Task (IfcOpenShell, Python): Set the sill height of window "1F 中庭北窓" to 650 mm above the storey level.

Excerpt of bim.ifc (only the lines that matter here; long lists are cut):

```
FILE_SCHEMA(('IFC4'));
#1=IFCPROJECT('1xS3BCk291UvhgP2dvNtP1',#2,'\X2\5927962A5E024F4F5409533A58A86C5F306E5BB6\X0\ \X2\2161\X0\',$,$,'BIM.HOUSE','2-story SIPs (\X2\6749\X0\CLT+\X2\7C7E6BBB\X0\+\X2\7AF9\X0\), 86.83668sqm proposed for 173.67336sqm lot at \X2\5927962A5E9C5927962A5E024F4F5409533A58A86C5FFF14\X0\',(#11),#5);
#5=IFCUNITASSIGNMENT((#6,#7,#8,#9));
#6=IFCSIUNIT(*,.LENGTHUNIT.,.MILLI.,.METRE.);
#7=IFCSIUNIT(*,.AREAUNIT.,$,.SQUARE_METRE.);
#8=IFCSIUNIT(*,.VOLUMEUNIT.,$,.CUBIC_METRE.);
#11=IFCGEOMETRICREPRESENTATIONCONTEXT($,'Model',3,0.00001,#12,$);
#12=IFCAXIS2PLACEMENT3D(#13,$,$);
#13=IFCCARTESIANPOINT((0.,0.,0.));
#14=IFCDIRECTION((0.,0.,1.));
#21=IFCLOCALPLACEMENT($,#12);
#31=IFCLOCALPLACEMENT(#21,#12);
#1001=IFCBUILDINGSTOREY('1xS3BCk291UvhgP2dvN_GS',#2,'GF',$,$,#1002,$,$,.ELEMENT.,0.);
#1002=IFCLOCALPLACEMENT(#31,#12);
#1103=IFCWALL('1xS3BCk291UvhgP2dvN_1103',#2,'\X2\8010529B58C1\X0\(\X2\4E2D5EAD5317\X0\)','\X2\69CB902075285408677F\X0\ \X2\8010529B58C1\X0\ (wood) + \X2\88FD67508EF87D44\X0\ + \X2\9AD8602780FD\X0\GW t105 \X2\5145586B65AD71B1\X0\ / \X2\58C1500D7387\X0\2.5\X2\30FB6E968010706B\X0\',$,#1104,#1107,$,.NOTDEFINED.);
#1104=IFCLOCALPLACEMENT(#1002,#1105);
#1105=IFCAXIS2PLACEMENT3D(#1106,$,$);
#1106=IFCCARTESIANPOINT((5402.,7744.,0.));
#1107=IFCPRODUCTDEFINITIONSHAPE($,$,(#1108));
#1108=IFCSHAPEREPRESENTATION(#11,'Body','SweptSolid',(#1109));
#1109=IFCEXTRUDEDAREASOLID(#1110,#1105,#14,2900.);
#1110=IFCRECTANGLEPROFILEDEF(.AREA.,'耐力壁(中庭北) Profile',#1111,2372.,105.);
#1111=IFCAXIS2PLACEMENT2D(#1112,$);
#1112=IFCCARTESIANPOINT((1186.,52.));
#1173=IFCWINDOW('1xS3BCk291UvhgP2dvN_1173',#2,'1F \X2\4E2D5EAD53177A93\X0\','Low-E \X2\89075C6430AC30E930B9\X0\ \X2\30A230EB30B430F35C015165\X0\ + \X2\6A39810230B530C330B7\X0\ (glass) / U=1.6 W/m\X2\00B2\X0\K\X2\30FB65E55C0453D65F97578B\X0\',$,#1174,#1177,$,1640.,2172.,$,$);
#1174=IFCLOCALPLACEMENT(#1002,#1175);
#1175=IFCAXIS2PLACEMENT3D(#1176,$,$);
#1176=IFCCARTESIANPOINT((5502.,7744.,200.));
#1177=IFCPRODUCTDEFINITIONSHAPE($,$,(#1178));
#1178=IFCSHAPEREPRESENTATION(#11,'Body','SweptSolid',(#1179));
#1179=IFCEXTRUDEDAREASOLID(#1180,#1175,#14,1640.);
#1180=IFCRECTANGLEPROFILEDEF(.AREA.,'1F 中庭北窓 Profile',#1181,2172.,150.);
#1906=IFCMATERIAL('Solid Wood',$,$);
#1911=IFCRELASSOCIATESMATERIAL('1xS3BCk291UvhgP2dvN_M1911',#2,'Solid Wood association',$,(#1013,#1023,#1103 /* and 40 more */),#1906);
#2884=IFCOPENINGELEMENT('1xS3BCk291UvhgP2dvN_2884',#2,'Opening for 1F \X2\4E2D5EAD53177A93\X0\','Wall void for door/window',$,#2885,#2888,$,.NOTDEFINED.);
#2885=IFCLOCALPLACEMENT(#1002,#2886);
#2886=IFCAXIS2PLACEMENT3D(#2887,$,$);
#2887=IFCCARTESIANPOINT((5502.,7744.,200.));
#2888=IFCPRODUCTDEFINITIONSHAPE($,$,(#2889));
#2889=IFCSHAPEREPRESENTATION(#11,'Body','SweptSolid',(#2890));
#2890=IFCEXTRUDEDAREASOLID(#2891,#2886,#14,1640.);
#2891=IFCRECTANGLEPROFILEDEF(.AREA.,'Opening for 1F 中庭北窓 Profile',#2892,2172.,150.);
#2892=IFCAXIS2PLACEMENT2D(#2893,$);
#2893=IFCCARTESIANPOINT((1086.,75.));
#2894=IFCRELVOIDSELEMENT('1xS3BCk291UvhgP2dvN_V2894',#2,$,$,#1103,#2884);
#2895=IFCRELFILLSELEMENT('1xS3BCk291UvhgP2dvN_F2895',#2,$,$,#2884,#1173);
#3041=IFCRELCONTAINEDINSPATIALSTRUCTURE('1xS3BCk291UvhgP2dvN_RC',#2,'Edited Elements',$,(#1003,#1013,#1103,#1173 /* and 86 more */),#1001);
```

```python
import numpy as np
import ifcopenshell
import ifcopenshell.api.geometry
import ifcopenshell.geom
import ifcopenshell.util.element
import ifcopenshell.util.placement
import ifcopenshell.util.shape
import ifcopenshell.util.unit

model = ifcopenshell.open("bim.ifc")
unit_scale = ifcopenshell.util.unit.calculate_unit_scale(model)

window = model.by_guid("1xS3BCk291UvhgP2dvN_1173")
opening = window.FillsVoids[0].RelatingOpeningElement
storey = ifcopenshell.util.element.get_container(window, ifc_class="IfcBuildingStorey")
level = ifcopenshell.util.placement.get_local_placement(storey.ObjectPlacement)[2, 3]

# The opening's origin need not be at the sill, so measure its lowest point.
shape = ifcopenshell.geom.create_shape(ifcopenshell.geom.settings(), opening)
bottom = ifcopenshell.util.shape.get_shape_bottom_elevation(shape, shape.geometry) / unit_scale
dz = level + 650.0 - bottom

shift = np.array([0.0, 0.0, dz])
# The window is not placed relative to its opening, so move both.
for product in (opening, window):
    matrix = ifcopenshell.util.placement.get_local_placement(product.ObjectPlacement)
    matrix[:3, 3] += shift
    ifcopenshell.api.geometry.edit_object_placement(model, product=product, matrix=matrix, is_si=False)

print(f"moved by {dz * unit_scale:+.3f} m")

model.write("bim-out.ifc")
```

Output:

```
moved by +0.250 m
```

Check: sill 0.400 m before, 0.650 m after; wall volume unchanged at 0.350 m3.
